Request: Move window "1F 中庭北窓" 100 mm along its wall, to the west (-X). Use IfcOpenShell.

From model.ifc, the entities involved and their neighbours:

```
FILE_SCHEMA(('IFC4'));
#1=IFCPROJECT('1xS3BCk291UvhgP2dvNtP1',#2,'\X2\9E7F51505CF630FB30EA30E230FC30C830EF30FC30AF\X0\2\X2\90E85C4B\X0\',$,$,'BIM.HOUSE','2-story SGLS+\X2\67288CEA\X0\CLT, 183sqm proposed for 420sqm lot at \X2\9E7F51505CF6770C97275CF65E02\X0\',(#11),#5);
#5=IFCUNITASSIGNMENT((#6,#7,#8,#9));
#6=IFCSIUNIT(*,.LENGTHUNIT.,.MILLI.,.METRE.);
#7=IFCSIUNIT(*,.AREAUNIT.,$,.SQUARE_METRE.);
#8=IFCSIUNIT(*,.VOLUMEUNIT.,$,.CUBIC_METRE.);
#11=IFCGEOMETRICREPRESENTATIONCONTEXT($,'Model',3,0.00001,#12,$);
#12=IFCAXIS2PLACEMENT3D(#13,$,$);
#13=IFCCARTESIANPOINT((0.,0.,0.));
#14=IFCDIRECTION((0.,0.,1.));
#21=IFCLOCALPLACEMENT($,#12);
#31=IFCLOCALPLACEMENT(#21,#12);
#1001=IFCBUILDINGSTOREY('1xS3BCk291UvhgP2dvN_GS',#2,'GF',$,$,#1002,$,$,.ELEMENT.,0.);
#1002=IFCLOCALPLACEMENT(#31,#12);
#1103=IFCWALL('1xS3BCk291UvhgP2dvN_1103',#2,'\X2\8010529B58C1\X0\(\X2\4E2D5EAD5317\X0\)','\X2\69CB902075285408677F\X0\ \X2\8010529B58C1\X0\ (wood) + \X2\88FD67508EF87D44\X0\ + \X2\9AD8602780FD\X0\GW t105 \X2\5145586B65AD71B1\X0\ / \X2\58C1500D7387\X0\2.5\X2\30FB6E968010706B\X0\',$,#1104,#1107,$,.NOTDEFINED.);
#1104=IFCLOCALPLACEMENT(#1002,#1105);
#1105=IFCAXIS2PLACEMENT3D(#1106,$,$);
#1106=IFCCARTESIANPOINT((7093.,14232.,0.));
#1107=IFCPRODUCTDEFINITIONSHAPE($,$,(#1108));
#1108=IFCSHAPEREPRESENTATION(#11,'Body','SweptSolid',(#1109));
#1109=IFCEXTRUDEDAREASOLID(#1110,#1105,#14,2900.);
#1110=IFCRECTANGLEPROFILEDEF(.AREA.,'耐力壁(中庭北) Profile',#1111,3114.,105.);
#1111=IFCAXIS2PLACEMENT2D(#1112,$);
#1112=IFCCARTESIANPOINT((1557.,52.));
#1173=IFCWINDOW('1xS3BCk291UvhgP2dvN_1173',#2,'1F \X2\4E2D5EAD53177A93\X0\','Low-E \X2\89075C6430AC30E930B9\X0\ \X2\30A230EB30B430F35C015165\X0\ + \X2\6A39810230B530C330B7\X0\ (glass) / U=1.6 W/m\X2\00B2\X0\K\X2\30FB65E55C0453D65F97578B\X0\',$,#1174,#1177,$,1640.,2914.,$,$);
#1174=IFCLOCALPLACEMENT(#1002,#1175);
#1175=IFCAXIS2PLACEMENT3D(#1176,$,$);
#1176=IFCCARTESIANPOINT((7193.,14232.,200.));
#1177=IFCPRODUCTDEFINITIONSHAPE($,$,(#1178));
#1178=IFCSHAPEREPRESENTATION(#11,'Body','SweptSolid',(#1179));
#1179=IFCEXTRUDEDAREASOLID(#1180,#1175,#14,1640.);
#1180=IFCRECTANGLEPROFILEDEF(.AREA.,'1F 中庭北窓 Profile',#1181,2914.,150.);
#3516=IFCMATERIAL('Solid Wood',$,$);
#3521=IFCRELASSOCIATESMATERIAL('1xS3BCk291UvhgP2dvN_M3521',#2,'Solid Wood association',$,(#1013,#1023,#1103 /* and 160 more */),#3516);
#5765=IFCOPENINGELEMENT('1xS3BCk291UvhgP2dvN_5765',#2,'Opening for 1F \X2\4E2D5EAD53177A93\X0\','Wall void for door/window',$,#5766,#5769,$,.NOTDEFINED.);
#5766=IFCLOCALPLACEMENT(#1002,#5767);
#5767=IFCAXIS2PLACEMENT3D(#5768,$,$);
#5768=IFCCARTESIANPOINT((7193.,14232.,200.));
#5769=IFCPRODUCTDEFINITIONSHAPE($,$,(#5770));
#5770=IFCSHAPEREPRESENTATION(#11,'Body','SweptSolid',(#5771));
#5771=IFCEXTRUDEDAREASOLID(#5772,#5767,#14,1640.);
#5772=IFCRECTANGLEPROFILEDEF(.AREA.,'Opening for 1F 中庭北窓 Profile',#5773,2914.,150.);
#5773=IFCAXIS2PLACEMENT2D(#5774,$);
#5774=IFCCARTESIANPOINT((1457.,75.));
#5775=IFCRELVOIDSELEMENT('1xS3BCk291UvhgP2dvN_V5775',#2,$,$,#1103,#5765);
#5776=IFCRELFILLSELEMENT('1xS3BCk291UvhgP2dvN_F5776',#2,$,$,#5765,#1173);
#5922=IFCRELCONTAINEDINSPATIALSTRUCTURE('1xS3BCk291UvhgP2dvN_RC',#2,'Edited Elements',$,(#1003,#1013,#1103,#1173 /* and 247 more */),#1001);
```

```python
import ifcopenshell
import ifcopenshell.api.geometry
import ifcopenshell.util.placement
import ifcopenshell.util.unit

model = ifcopenshell.open("model.ifc")
unit_scale = ifcopenshell.util.unit.calculate_unit_scale(model)

window = model.by_guid("1xS3BCk291UvhgP2dvN_1173")
opening = window.FillsVoids[0].RelatingOpeningElement
wall = opening.VoidsElements[0].RelatingBuildingElement

wall_matrix = ifcopenshell.util.placement.get_local_placement(wall.ObjectPlacement)
shift = wall_matrix[:3, 0] * -0.1 / unit_scale
before = ifcopenshell.util.placement.get_local_placement(window.ObjectPlacement)[:3, 3].copy()

# The window is not placed relative to its opening, so move both.
for product in (opening, window):
    matrix = ifcopenshell.util.placement.get_local_placement(product.ObjectPlacement)
    matrix[:3, 3] += shift
    ifcopenshell.api.geometry.edit_object_placement(model, product=product, matrix=matrix, is_si=False)

after = ifcopenshell.util.placement.get_local_placement(window.ObjectPlacement)[:3, 3]
print("window moved by", (after - before).round(3) + 0.0)

model.write("model_v2.ifc")
```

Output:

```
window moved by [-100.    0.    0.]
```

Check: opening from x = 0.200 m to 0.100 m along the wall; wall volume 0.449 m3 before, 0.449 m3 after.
